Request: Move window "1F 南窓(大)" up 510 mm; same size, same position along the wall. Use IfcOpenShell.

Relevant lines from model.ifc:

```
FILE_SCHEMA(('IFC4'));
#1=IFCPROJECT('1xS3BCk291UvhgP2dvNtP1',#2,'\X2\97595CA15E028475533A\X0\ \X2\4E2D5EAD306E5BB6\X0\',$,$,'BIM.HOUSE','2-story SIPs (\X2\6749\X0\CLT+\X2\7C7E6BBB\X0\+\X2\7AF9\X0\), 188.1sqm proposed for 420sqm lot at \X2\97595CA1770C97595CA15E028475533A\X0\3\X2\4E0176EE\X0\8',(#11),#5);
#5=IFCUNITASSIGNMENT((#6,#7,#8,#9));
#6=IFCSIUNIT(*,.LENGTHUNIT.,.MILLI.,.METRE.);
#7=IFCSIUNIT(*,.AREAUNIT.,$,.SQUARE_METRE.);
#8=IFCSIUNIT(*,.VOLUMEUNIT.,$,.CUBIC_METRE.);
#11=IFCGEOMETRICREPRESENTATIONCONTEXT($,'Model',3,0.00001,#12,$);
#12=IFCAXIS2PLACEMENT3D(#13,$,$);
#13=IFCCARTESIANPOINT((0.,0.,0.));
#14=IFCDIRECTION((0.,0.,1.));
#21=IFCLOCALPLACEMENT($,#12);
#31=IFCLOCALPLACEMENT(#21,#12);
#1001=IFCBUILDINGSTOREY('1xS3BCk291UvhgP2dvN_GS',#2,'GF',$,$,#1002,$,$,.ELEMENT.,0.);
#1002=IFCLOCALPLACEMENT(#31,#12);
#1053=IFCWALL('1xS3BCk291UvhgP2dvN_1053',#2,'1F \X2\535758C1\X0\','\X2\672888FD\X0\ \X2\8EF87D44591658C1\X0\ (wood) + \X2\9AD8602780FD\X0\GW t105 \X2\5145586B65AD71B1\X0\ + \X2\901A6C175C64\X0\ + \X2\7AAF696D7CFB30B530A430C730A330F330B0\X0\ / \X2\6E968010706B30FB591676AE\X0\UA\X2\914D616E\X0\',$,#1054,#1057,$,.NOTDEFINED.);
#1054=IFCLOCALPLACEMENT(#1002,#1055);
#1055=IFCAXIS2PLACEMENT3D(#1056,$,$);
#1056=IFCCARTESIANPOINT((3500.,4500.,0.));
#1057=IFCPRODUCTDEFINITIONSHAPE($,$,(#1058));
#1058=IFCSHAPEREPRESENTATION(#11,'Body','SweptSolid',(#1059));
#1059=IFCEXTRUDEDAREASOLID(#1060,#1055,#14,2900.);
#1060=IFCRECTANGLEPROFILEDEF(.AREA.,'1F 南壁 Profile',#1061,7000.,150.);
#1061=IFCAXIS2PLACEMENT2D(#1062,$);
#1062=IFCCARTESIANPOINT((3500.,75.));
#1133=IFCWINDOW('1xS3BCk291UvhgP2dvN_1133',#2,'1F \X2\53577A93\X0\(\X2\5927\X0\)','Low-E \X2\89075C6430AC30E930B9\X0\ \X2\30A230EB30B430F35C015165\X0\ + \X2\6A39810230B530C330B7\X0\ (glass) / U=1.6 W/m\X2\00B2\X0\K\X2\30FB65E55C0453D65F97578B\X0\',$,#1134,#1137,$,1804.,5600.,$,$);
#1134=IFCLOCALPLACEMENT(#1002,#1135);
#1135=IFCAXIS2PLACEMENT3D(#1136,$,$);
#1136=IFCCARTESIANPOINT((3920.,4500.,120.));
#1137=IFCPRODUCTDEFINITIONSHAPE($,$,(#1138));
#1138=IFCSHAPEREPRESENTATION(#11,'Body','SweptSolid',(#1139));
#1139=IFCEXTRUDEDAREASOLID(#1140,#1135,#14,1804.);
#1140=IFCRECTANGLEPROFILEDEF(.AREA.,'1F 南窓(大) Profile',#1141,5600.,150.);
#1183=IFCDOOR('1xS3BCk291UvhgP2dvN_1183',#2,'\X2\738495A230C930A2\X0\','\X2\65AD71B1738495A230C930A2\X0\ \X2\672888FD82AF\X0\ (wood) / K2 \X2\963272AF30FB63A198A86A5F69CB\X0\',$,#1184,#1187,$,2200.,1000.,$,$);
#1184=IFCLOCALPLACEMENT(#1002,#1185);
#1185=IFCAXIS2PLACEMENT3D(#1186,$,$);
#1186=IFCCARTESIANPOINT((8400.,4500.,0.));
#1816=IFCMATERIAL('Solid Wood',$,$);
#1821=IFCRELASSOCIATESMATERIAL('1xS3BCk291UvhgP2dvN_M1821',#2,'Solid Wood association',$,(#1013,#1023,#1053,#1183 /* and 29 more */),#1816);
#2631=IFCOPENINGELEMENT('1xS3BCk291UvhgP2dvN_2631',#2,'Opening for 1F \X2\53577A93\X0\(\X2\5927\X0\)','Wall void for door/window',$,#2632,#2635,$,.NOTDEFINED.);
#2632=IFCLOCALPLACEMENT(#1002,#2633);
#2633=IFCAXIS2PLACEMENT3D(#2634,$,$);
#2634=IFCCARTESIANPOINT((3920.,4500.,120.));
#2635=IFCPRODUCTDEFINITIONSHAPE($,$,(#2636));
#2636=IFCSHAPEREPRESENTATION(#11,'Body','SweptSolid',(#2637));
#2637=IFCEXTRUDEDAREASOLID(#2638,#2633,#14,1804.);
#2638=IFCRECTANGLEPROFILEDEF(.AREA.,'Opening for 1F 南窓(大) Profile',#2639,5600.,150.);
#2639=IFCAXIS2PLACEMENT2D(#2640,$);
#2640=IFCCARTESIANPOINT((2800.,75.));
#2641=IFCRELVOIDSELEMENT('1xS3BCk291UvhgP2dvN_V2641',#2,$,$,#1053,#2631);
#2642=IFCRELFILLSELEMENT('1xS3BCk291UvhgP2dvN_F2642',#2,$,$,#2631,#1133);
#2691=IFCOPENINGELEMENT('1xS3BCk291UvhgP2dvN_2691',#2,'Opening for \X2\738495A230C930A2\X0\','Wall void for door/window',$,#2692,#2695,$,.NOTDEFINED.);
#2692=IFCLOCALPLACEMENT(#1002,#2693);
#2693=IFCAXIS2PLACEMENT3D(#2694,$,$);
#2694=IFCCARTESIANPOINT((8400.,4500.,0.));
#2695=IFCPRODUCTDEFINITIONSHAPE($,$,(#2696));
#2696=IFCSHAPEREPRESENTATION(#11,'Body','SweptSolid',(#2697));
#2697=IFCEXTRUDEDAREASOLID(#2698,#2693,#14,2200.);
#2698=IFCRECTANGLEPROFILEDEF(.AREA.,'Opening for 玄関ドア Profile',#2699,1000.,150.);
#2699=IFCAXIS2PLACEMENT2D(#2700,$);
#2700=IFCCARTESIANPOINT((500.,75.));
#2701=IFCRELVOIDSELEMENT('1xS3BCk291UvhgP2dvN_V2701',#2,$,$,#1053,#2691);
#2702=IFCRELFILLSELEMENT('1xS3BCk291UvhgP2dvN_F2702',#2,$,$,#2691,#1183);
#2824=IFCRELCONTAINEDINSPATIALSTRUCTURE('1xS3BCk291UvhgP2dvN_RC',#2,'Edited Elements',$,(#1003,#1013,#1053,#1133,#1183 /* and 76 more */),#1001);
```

```python
import numpy as np
import ifcopenshell
import ifcopenshell.api.geometry
import ifcopenshell.util.placement
import ifcopenshell.util.unit

model = ifcopenshell.open("model.ifc")
unit_scale = ifcopenshell.util.unit.calculate_unit_scale(model)

window = model.by_guid("1xS3BCk291UvhgP2dvN_1133")
opening = window.FillsVoids[0].RelatingOpeningElement
dz = 0.51 / unit_scale

shift = np.array([0.0, 0.0, dz])
# The window is not placed relative to its opening, so move both.
for product in (opening, window):
    matrix = ifcopenshell.util.placement.get_local_placement(product.ObjectPlacement)
    matrix[:3, 3] += shift
    ifcopenshell.api.geometry.edit_object_placement(model, product=product, matrix=matrix, is_si=False)

print(f"moved by {dz * unit_scale:+.3f} m")

model.write("model-out.ifc")
```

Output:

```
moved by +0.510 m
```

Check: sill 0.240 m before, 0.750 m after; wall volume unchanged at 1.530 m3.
